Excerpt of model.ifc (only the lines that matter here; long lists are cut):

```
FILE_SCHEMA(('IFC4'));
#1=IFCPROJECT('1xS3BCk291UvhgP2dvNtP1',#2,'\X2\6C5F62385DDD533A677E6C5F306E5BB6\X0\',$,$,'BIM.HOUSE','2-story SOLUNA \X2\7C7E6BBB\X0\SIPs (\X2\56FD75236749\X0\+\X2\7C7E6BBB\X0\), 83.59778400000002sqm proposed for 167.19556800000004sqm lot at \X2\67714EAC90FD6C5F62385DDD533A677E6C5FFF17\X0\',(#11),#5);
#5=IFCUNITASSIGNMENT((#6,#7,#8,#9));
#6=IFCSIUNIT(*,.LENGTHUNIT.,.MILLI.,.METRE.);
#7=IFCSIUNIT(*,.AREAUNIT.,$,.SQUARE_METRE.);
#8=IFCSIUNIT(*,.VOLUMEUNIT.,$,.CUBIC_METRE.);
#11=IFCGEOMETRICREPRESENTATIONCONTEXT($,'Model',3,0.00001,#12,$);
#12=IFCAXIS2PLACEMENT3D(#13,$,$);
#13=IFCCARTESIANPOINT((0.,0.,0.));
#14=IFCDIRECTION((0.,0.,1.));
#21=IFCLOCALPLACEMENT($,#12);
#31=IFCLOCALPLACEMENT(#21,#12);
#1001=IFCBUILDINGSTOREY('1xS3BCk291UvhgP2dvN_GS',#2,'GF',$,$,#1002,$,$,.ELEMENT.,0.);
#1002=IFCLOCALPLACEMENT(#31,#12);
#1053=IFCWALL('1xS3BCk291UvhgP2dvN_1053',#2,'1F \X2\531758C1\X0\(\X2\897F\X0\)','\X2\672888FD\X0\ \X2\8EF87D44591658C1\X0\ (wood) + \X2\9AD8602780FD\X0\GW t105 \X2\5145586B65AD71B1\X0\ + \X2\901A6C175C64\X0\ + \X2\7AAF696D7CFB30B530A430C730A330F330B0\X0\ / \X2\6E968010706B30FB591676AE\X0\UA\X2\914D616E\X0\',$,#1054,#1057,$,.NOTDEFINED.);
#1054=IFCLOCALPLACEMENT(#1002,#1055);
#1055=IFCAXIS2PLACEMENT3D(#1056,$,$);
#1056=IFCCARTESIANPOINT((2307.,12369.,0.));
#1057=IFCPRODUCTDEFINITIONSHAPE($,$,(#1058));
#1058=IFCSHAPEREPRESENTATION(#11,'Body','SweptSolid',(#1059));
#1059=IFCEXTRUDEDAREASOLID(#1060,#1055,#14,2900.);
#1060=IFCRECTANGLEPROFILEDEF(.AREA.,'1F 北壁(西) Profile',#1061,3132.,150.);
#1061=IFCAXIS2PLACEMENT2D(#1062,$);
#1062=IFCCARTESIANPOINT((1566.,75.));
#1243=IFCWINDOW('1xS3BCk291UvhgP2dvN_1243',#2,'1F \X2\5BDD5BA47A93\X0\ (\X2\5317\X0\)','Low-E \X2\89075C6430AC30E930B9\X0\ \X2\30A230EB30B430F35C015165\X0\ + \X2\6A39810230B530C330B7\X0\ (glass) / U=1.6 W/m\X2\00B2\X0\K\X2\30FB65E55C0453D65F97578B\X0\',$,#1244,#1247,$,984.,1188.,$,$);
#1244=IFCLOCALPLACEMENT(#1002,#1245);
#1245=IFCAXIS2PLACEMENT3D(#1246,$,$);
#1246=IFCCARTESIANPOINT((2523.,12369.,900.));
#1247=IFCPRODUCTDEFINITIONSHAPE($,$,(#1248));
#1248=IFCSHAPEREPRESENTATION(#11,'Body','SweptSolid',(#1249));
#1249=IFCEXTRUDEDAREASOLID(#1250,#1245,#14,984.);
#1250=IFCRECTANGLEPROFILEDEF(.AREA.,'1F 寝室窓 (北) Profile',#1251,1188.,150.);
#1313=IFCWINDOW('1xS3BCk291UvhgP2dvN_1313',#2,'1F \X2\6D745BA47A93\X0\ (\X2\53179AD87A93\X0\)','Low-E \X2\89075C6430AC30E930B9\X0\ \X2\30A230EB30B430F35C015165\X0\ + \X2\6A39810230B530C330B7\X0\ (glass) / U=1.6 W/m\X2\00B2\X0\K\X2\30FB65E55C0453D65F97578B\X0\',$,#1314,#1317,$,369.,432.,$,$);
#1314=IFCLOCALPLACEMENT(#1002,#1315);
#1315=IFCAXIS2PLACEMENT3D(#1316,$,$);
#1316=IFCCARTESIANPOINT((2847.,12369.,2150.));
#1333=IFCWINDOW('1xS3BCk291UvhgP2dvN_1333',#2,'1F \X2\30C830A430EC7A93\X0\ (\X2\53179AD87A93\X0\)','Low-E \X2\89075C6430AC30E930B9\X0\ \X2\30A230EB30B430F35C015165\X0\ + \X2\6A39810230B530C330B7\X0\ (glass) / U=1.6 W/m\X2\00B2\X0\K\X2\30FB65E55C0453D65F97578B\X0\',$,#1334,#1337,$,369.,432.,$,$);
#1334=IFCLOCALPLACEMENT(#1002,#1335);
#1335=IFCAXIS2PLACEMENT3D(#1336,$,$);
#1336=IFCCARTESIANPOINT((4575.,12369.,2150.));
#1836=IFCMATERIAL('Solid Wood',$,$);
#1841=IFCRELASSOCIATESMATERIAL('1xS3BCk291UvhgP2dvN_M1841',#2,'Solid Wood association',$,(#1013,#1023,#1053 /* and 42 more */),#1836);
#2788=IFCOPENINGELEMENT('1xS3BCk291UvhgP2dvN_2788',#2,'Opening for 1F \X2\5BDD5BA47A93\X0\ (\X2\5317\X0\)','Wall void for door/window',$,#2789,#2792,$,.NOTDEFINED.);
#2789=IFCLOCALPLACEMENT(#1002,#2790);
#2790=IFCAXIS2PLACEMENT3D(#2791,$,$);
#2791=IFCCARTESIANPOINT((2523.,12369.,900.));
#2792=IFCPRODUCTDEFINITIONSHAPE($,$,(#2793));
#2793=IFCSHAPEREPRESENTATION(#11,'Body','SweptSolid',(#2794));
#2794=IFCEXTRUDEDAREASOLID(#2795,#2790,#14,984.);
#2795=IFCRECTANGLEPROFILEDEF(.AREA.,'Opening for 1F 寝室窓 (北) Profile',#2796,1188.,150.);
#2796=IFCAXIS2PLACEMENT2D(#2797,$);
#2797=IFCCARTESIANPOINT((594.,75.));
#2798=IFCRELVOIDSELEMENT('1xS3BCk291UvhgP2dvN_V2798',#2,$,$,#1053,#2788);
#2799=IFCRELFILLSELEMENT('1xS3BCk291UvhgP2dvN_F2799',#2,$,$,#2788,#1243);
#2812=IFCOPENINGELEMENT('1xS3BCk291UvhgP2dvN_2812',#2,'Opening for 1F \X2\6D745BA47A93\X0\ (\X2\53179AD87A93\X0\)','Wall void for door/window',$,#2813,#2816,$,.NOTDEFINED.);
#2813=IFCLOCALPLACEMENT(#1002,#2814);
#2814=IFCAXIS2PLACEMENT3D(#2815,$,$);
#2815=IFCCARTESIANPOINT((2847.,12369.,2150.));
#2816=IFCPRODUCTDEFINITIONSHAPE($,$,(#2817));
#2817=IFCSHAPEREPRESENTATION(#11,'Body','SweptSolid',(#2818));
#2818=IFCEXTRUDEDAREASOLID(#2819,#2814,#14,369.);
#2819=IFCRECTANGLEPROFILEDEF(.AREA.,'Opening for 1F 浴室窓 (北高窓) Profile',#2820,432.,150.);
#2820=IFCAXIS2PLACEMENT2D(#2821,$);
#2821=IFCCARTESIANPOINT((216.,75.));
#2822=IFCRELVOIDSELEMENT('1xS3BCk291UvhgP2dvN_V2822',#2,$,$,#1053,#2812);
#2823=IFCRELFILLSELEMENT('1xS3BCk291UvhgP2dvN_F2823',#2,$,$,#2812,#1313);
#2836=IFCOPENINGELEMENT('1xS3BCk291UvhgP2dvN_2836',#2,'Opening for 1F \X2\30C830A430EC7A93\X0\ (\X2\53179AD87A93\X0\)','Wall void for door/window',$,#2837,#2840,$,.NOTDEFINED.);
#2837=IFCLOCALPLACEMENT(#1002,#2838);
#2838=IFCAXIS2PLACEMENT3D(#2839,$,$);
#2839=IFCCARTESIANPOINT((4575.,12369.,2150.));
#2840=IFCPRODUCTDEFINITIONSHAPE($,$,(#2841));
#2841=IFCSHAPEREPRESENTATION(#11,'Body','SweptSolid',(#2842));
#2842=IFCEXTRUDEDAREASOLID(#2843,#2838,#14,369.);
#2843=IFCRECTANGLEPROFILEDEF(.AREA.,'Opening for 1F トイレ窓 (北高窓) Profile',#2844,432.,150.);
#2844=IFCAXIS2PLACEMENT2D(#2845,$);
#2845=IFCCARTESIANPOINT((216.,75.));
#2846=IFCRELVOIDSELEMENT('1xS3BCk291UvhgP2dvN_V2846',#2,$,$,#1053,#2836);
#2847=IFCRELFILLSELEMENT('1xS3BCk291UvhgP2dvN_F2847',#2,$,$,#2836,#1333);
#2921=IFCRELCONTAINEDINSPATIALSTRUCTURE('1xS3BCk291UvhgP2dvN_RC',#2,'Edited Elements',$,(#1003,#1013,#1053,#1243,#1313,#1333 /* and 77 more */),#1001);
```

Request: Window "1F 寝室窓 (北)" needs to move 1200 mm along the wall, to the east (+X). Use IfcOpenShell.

```python
import ifcopenshell
import ifcopenshell.api.geometry
import ifcopenshell.util.placement
import ifcopenshell.util.unit

model = ifcopenshell.open("model.ifc")
unit_scale = ifcopenshell.util.unit.calculate_unit_scale(model)

window = model.by_guid("1xS3BCk291UvhgP2dvN_1243")
opening = window.FillsVoids[0].RelatingOpeningElement
wall = opening.VoidsElements[0].RelatingBuildingElement

wall_matrix = ifcopenshell.util.placement.get_local_placement(wall.ObjectPlacement)
shift = wall_matrix[:3, 0] * 1.2 / unit_scale
before = ifcopenshell.util.placement.get_local_placement(window.ObjectPlacement)[:3, 3].copy()

# The window is not placed relative to its opening, so move both.
for product in (opening, window):
    matrix = ifcopenshell.util.placement.get_local_placement(product.ObjectPlacement)
    matrix[:3, 3] += shift
    ifcopenshell.api.geometry.edit_object_placement(model, product=product, matrix=matrix, is_si=False)

after = ifcopenshell.util.placement.get_local_placement(window.ObjectPlacement)[:3, 3]
print("window moved by", (after - before).round(3) + 0.0)

model.write("model_rev.ifc")
```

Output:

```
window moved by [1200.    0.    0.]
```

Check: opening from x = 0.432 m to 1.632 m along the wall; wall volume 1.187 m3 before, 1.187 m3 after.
